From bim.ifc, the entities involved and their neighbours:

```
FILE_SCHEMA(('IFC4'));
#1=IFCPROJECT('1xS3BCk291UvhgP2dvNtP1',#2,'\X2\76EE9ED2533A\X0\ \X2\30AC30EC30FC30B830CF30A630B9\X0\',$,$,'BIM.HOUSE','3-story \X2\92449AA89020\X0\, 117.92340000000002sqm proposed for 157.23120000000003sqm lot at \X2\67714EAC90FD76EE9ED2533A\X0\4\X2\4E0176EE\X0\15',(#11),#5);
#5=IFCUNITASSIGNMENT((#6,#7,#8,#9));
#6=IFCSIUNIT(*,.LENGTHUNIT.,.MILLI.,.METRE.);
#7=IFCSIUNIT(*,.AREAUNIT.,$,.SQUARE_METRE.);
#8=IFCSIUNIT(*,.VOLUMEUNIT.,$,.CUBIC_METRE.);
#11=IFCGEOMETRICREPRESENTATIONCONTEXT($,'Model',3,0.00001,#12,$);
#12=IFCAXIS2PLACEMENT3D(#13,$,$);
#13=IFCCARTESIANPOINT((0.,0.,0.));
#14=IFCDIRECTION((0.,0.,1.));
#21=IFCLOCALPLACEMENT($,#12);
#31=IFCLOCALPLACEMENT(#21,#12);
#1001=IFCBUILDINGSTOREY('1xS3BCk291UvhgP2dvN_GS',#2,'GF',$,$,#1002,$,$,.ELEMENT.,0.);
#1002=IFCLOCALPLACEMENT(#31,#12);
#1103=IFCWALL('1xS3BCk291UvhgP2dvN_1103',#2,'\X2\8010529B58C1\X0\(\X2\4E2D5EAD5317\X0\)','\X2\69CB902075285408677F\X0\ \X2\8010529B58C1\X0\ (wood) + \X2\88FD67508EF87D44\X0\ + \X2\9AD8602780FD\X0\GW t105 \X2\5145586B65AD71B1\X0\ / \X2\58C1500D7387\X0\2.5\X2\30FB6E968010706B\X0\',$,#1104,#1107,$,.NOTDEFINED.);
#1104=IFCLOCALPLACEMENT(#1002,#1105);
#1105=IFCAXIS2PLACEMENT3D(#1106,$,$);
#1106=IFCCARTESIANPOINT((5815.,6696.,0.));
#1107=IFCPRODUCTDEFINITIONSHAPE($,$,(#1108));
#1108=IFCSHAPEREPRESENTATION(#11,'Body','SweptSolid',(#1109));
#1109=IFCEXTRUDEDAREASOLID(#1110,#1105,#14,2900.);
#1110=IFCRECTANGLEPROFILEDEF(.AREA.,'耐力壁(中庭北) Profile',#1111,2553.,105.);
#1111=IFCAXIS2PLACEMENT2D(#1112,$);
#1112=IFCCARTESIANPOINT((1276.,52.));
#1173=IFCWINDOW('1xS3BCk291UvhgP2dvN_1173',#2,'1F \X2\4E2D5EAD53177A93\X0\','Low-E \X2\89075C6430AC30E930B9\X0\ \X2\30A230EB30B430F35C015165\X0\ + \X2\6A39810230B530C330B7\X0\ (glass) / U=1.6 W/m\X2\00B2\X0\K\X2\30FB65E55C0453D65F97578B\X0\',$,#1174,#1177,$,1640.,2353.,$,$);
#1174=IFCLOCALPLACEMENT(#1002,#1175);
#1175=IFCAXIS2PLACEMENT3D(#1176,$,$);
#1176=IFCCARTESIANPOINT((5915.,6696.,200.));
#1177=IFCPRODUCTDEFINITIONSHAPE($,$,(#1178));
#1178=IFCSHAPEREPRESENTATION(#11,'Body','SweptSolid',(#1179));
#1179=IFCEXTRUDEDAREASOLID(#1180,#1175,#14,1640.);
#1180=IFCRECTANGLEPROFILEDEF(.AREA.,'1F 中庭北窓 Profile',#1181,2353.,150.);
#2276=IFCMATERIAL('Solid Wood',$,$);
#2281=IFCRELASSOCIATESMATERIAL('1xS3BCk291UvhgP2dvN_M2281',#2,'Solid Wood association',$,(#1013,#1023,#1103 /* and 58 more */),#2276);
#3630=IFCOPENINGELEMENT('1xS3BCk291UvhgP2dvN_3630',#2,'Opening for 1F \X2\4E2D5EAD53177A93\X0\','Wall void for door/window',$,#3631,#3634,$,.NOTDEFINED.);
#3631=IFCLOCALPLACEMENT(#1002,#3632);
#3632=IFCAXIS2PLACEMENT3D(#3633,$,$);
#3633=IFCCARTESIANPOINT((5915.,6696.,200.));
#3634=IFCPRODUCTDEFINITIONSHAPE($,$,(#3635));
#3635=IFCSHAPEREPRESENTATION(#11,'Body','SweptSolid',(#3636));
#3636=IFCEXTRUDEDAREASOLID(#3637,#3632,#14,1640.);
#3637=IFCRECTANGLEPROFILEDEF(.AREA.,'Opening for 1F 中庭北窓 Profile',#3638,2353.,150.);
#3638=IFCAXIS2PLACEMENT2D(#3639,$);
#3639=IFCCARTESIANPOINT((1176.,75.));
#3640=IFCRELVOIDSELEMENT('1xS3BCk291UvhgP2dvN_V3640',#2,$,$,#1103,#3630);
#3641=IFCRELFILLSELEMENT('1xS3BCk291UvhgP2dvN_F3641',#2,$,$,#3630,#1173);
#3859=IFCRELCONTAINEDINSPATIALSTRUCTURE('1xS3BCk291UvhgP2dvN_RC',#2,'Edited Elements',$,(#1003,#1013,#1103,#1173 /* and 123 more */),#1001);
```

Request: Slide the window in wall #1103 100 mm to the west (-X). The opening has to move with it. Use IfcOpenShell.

```python
import ifcopenshell
import ifcopenshell.api.geometry
import ifcopenshell.util.placement
import ifcopenshell.util.unit

model = ifcopenshell.open("bim.ifc")
unit_scale = ifcopenshell.util.unit.calculate_unit_scale(model)

window = model.by_guid("1xS3BCk291UvhgP2dvN_1173")
opening = window.FillsVoids[0].RelatingOpeningElement
wall = opening.VoidsElements[0].RelatingBuildingElement

wall_matrix = ifcopenshell.util.placement.get_local_placement(wall.ObjectPlacement)
shift = wall_matrix[:3, 0] * -0.1 / unit_scale
before = ifcopenshell.util.placement.get_local_placement(window.ObjectPlacement)[:3, 3].copy()

# The window is not placed relative to its opening, so move both.
for product in (opening, window):
    matrix = ifcopenshell.util.placement.get_local_placement(product.ObjectPlacement)
    matrix[:3, 3] += shift
    ifcopenshell.api.geometry.edit_object_placement(model, product=product, matrix=matrix, is_si=False)

after = ifcopenshell.util.placement.get_local_placement(window.ObjectPlacement)[:3, 3]
print("window moved by", (after - before).round(3) + 0.0)

model.write("bim_rev.ifc")
```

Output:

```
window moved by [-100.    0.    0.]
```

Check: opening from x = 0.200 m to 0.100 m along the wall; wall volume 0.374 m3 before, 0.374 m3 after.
